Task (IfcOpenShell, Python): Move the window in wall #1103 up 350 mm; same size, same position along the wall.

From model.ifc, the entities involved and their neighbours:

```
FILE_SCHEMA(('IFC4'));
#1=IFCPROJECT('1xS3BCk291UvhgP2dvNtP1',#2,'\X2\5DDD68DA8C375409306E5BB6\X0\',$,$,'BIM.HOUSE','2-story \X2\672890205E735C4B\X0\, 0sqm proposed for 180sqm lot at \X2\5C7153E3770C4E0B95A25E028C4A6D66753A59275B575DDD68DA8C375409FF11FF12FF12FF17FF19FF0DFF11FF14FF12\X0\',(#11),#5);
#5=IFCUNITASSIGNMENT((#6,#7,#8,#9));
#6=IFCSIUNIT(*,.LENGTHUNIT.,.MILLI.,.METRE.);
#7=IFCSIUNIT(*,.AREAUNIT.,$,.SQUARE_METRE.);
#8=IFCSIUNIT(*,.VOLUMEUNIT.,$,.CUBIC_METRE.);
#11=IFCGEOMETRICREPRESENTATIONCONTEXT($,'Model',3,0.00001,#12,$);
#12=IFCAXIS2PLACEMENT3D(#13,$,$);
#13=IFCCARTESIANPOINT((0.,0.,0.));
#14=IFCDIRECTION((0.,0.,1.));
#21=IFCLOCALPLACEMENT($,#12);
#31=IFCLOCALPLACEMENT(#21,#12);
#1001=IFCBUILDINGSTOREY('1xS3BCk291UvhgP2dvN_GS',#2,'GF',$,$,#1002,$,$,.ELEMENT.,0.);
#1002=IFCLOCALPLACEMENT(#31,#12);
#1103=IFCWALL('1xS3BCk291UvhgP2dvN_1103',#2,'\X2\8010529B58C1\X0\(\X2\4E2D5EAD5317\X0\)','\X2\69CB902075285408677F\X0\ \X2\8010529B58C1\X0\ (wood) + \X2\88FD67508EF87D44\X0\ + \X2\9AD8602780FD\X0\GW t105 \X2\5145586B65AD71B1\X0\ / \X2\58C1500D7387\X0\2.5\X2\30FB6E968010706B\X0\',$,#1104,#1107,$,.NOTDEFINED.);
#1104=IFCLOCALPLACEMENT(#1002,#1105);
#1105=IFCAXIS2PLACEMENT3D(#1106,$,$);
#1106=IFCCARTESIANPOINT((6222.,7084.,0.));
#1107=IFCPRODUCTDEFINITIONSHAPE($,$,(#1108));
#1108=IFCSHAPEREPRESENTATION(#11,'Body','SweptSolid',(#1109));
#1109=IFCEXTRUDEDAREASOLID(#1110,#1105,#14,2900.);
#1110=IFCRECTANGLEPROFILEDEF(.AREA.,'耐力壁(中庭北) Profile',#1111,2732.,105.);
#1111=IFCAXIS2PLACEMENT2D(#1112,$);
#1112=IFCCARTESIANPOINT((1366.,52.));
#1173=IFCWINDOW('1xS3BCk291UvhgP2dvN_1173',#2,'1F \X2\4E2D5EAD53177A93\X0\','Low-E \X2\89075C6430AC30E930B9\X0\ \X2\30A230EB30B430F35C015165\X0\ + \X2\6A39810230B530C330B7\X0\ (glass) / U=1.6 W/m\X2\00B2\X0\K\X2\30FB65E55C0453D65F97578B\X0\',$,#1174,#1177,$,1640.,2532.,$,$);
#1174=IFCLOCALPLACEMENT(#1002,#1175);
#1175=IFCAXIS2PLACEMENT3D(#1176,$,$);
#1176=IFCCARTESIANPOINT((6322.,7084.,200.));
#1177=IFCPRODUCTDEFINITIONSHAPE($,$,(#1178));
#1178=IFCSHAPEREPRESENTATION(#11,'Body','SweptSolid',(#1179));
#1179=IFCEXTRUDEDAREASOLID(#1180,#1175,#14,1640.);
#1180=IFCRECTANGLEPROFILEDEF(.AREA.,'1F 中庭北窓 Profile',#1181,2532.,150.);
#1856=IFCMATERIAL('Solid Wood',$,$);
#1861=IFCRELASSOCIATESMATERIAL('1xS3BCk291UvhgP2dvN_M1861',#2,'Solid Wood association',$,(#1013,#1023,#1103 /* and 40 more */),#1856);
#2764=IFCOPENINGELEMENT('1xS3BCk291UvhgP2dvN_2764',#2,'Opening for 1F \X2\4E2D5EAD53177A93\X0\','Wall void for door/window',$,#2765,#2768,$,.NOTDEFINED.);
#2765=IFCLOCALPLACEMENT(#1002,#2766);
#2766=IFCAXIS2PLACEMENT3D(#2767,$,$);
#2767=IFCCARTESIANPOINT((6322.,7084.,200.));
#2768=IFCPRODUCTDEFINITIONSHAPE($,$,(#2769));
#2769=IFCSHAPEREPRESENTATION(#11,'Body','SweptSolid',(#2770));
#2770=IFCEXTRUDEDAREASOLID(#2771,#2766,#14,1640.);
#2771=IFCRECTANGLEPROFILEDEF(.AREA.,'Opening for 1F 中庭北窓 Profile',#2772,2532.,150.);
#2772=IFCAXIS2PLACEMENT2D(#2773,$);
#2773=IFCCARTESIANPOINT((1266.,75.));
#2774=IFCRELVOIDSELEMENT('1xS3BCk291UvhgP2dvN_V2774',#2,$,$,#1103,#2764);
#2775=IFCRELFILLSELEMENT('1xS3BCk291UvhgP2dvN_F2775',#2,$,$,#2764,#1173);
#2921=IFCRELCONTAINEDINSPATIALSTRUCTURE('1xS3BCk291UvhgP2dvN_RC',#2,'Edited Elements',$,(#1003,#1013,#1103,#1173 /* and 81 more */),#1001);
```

```python
import numpy as np
import ifcopenshell
import ifcopenshell.api.geometry
import ifcopenshell.util.placement
import ifcopenshell.util.unit

model = ifcopenshell.open("model.ifc")
unit_scale = ifcopenshell.util.unit.calculate_unit_scale(model)

window = model.by_id(1173)
opening = window.FillsVoids[0].RelatingOpeningElement
dz = 0.35 / unit_scale

shift = np.array([0.0, 0.0, dz])
# The window is not placed relative to its opening, so move both.
for product in (opening, window):
    matrix = ifcopenshell.util.placement.get_local_placement(product.ObjectPlacement)
    matrix[:3, 3] += shift
    ifcopenshell.api.geometry.edit_object_placement(model, product=product, matrix=matrix, is_si=False)

print(f"moved by {dz * unit_scale:+.3f} m")

model.write("model-out.ifc")
```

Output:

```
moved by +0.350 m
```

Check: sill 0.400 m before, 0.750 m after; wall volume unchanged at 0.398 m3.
